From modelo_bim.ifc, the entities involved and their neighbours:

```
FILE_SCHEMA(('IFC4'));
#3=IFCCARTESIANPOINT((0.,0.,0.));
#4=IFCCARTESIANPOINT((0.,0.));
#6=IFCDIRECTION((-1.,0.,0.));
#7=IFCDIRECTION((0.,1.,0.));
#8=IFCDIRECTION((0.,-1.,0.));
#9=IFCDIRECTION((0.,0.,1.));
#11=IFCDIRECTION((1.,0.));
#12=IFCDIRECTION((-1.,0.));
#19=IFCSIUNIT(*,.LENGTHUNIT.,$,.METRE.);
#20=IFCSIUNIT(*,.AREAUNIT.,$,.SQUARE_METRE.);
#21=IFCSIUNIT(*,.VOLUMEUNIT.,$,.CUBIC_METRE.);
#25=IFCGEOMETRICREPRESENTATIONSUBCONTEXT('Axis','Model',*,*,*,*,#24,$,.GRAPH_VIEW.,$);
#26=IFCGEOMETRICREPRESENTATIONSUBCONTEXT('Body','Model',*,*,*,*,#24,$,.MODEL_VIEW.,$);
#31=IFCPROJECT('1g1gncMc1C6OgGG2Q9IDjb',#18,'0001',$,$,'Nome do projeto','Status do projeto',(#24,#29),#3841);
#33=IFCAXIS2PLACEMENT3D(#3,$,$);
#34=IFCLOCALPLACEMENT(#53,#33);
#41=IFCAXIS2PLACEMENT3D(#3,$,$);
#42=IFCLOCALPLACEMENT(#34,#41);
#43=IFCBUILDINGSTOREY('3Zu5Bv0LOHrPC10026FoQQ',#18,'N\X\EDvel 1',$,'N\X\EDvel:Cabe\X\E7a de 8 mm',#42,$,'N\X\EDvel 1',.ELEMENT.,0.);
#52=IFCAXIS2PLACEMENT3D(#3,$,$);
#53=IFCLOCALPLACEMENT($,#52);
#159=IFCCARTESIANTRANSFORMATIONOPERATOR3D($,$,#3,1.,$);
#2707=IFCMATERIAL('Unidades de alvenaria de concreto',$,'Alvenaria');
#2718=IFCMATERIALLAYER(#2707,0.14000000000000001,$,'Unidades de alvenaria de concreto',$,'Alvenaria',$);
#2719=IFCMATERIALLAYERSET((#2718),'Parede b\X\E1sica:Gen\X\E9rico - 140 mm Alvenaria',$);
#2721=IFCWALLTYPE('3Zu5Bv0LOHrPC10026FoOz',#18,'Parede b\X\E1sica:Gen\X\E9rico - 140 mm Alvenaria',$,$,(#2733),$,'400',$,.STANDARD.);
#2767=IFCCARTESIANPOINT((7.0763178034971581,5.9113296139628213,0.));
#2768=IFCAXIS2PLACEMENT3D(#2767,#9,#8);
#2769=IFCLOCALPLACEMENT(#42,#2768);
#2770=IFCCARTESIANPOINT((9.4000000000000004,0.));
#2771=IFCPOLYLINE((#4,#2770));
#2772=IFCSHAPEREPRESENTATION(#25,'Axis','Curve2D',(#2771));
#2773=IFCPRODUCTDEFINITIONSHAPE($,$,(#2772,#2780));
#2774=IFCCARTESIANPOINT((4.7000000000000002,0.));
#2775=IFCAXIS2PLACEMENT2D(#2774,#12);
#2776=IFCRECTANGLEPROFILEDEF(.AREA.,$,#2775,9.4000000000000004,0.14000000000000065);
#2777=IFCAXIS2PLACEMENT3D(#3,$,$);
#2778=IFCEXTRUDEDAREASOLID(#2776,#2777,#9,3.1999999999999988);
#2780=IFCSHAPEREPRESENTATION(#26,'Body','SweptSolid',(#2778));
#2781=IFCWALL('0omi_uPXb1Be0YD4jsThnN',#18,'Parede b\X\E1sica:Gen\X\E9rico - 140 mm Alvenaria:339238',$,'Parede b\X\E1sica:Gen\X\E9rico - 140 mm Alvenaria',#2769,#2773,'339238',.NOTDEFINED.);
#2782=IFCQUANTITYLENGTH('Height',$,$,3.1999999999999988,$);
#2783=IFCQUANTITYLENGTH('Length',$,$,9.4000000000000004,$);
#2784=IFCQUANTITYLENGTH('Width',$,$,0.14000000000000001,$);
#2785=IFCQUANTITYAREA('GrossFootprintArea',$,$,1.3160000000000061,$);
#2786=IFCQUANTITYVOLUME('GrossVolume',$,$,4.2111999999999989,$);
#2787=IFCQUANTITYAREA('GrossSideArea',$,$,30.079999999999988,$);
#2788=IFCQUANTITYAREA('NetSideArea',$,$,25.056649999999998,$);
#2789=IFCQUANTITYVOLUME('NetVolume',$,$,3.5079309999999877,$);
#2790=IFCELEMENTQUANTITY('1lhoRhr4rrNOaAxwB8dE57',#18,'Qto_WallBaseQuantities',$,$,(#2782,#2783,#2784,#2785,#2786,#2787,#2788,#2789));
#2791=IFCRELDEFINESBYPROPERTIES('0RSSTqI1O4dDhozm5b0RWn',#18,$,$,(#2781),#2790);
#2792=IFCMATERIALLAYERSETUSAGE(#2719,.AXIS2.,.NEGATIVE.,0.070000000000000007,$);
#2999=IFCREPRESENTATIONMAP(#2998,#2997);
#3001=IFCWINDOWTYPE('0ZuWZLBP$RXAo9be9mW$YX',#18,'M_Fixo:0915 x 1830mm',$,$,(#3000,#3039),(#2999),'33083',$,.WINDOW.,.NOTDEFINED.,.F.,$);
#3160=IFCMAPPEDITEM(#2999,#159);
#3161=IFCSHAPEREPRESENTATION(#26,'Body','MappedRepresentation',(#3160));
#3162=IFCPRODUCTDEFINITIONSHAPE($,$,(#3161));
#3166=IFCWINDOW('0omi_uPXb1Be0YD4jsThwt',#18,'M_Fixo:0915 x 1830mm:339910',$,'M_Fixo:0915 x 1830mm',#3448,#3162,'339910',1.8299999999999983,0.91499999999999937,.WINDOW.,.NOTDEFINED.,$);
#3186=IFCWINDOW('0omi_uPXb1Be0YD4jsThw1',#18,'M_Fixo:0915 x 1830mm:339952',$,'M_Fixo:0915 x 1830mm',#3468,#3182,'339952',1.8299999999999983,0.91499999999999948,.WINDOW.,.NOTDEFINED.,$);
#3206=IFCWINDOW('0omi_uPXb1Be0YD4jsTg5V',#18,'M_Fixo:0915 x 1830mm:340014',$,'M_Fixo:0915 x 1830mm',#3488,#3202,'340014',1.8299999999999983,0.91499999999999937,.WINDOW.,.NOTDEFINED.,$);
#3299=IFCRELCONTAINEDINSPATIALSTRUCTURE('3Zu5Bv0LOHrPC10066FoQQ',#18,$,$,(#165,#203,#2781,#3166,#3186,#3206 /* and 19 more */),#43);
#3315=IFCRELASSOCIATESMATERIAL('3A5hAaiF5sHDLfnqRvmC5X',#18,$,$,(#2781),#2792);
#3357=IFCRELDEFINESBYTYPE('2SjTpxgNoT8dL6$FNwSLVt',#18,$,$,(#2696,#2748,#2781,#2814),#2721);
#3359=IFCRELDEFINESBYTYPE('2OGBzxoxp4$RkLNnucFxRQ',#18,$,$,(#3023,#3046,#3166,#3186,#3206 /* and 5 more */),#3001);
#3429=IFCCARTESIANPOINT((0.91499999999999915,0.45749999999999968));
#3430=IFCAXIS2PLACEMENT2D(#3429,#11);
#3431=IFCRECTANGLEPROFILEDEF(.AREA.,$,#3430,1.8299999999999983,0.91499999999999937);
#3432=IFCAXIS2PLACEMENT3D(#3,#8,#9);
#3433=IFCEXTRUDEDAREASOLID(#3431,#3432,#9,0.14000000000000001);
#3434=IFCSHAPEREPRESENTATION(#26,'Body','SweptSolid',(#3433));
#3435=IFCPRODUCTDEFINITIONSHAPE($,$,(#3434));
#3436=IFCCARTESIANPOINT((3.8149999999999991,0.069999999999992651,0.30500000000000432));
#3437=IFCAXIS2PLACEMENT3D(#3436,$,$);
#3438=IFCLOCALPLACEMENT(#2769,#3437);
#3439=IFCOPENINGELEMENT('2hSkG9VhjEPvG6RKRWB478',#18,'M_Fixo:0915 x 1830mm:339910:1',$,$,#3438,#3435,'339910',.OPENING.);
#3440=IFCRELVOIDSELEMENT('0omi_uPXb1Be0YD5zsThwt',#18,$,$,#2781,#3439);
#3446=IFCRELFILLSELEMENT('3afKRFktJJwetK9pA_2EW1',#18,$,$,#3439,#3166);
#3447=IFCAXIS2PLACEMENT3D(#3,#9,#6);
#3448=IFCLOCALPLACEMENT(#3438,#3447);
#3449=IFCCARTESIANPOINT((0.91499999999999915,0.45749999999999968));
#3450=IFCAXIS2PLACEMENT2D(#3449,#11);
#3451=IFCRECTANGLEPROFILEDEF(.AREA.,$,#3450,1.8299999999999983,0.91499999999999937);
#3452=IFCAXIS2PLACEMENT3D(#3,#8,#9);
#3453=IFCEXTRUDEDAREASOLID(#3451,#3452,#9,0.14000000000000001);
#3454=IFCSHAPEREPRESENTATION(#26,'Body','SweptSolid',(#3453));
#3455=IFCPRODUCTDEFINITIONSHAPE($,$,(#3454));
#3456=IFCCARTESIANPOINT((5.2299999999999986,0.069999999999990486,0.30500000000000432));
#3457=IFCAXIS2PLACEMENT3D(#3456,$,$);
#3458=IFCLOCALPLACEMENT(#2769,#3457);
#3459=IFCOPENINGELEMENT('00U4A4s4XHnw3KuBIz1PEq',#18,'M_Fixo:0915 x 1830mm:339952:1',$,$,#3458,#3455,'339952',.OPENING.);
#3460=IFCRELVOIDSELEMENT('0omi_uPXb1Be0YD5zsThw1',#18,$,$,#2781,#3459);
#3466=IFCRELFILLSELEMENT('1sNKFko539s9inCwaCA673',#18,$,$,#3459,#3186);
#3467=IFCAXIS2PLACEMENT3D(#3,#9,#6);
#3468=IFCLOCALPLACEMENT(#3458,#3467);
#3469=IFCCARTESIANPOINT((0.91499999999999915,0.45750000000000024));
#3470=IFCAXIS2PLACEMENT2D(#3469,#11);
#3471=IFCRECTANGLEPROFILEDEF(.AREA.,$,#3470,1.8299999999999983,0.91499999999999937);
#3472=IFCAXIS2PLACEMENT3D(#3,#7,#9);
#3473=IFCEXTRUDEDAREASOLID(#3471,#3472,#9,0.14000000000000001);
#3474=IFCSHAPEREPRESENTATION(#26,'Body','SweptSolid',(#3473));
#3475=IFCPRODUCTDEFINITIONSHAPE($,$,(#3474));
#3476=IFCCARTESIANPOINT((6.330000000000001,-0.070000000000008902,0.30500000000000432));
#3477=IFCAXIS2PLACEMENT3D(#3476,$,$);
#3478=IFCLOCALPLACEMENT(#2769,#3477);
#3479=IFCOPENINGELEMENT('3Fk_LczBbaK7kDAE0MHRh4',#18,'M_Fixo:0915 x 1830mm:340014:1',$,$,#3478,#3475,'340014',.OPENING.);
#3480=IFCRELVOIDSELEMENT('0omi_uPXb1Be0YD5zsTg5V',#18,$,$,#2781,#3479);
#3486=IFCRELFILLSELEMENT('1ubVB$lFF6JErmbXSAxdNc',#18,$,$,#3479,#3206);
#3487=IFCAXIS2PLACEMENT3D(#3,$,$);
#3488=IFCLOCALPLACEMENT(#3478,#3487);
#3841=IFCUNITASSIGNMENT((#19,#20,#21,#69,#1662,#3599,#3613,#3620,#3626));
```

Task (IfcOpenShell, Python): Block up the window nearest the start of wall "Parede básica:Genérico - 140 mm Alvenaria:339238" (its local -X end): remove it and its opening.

```python
import ifcopenshell
import ifcopenshell.api.feature
import ifcopenshell.api.pset
import ifcopenshell.api.root
import ifcopenshell.geom
import ifcopenshell.util.element
import ifcopenshell.util.shape
import ifcopenshell.util.unit

model = ifcopenshell.open("modelo_bim.ifc")
area_scale = ifcopenshell.util.unit.calculate_unit_scale(model, "AREAUNIT")
volume_scale = ifcopenshell.util.unit.calculate_unit_scale(model, "VOLUMEUNIT")
settings = ifcopenshell.geom.settings()


def volume(element):
    """Net volume in cubic metres, openings subtracted."""
    shape = ifcopenshell.geom.create_shape(settings, element)
    return ifcopenshell.util.shape.get_volume(shape.geometry)


window = model.by_guid("0omi_uPXb1Be0YD4jsThwt")
opening = window.FillsVoids[0].RelatingOpeningElement
wall = opening.VoidsElements[0].RelatingBuildingElement
before = volume(wall)

ifcopenshell.api.root.remove_product(model, product=window)
ifcopenshell.api.feature.remove_feature(model, feature=opening)

after = volume(wall)
thickness = 0.14  # wall thickness in metres

# Update the wall's stored quantities.
qto = model.by_id(ifcopenshell.util.element.get_pset(wall, "Qto_WallBaseQuantities", should_inherit=False)["id"])
ifcopenshell.api.pset.edit_qto(model, qto=qto, properties={
    "NetSideArea": after / thickness / area_scale,
    "NetVolume": after / volume_scale,
})

print(f"wall volume {before:.3f} -> {after:.3f} m3")

model.write("modelo_bim_edited.ifc")
```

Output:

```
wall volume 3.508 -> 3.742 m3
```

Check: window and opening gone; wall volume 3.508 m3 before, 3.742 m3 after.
